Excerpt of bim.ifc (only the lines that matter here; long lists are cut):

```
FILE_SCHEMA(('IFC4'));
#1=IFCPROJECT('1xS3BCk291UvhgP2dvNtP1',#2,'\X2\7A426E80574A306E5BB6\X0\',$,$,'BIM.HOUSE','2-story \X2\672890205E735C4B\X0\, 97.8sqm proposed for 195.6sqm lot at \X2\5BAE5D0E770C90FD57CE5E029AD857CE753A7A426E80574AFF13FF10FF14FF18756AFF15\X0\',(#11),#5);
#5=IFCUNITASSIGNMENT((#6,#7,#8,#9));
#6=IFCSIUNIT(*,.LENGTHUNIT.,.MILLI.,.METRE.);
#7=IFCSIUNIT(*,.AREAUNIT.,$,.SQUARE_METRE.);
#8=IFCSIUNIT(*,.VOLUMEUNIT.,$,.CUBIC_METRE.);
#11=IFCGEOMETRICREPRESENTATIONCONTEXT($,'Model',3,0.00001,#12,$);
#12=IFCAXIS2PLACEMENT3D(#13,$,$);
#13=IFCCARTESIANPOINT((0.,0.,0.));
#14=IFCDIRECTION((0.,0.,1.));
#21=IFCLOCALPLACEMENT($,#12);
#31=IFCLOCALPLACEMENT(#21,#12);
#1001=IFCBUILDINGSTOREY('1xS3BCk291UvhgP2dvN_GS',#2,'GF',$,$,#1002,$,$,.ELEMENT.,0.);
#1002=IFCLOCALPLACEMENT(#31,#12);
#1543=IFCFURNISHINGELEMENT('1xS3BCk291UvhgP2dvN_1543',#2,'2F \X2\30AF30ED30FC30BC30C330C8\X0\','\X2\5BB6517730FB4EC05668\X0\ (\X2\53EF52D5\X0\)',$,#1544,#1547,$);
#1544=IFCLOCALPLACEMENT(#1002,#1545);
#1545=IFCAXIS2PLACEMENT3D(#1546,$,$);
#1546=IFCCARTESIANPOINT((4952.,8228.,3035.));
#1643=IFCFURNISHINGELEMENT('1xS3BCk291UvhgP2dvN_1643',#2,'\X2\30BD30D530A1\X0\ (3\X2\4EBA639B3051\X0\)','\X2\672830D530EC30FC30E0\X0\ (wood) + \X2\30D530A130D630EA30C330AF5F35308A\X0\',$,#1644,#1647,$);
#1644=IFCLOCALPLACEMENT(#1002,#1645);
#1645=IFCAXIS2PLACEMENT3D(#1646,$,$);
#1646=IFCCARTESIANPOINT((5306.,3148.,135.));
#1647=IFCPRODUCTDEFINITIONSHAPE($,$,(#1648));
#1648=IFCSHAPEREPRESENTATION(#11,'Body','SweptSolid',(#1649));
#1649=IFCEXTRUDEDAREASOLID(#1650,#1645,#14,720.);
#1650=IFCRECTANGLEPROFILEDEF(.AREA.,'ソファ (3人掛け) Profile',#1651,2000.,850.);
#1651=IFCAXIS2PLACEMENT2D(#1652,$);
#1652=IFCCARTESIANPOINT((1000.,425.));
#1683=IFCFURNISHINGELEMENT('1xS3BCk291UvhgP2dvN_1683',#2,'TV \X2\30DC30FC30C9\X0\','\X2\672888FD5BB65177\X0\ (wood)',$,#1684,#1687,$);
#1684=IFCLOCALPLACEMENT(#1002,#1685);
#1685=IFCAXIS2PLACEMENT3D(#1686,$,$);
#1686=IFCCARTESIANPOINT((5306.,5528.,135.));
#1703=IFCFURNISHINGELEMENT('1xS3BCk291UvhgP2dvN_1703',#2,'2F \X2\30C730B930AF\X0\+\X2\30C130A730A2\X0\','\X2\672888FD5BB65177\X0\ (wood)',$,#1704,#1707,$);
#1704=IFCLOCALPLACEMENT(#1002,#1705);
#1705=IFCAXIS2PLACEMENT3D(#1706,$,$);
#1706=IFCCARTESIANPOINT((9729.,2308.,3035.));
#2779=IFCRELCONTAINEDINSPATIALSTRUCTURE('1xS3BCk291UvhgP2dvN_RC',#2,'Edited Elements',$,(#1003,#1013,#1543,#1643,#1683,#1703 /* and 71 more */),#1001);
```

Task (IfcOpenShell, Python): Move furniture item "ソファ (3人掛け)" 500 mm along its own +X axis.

```python
import ifcopenshell
import ifcopenshell.api.geometry
import ifcopenshell.util.placement
import ifcopenshell.util.unit

model = ifcopenshell.open("bim.ifc")
unit_scale = ifcopenshell.util.unit.calculate_unit_scale(model)

item = model.by_guid("1xS3BCk291UvhgP2dvN_1643")
matrix = ifcopenshell.util.placement.get_local_placement(item.ObjectPlacement)
matrix[:3, 3] += matrix[:3, 0] * 0.5 / unit_scale
ifcopenshell.api.geometry.edit_object_placement(model, product=item, matrix=matrix, is_si=False)

print(ifcopenshell.util.placement.get_local_placement(item.ObjectPlacement).round(3) + 0.0)

model.write("bim_v2.ifc")
```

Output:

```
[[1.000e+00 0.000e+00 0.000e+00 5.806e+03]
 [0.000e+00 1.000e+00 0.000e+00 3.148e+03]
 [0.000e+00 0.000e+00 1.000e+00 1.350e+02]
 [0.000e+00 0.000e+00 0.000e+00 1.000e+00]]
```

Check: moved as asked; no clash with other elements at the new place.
